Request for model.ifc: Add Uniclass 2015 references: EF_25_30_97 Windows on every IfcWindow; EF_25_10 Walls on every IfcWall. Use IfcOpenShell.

First a look at what the model holds.

```python
import ifcopenshell

model = ifcopenshell.open("model.ifc")
print(model.schema)
print("classifications:", [c.Name for c in model.by_type("IfcClassification")])
for ifc_class in ("IfcDoor", "IfcRoof", "IfcStair", "IfcWall", "IfcWindow"):
    print(ifc_class, len(model.by_type(ifc_class)))
```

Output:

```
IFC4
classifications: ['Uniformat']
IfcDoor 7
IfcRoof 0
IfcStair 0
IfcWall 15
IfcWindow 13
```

```python
import ifcopenshell
import ifcopenshell.api.classification

model = ifcopenshell.open("model.ifc")

system = ifcopenshell.api.classification.add_classification(model, classification="Uniclass 2015")

codes = {
    "IfcWindow": ("EF_25_30_97", "Windows"),
    "IfcWall": ("EF_25_10", "Walls"),
}
for ifc_class, (code, name) in codes.items():
    products = model.by_type(ifc_class)
    ifcopenshell.api.classification.add_reference(
        model, products=products, classification=system, identification=code, name=name
    )
    print(code, len(products))

model.write("model_rev.ifc")
```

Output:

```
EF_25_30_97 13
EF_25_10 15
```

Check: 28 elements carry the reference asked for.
